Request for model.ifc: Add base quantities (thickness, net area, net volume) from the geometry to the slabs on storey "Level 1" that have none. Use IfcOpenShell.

First a look at what the model holds.

```python
import ifcopenshell
import ifcopenshell.util.element
import ifcopenshell.util.unit

model = ifcopenshell.open("model.ifc")
print(model.schema)
for unit_type in ("LENGTHUNIT", "AREAUNIT", "VOLUMEUNIT"):
    print(unit_type, ifcopenshell.util.unit.calculate_unit_scale(model, unit_type))
storey = next(s for s in model.by_type("IfcBuildingStorey") if s.Name == "Level 1")
slabs = [e for e in ifcopenshell.util.element.get_decomposition(storey) if e.is_a("IfcSlab")]
for e in sorted(slabs, key=lambda e: e.id()):
    print(e.id(), e.is_a(), e.Name, list(ifcopenshell.util.element.get_psets(e, qtos_only=True)), sep=" | ")
```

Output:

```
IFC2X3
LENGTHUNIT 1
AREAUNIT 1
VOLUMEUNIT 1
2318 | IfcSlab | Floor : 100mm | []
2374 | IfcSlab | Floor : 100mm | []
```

```python
import ifcopenshell
import ifcopenshell.api.pset
import ifcopenshell.geom
import ifcopenshell.util.element
import ifcopenshell.util.shape
import ifcopenshell.util.unit

model = ifcopenshell.open("model.ifc")
unit_scale = ifcopenshell.util.unit.calculate_unit_scale(model)
area_scale = ifcopenshell.util.unit.calculate_unit_scale(model, "AREAUNIT")
volume_scale = ifcopenshell.util.unit.calculate_unit_scale(model, "VOLUMEUNIT")
settings = ifcopenshell.geom.settings()

storey = next(s for s in model.by_type("IfcBuildingStorey") if s.Name == "Level 1")
slabs = [e for e in ifcopenshell.util.element.get_decomposition(storey) if e.is_a("IfcSlab")]

for e in sorted(slabs, key=lambda e: e.id()):
    if ifcopenshell.util.element.get_psets(e, qtos_only=True, should_inherit=False):
        continue
    # Geometry comes back in metres, in the element's own axes.
    shape = ifcopenshell.geom.create_shape(settings, e)
    values = {
        "Width": ifcopenshell.util.shape.get_z(shape.geometry) / unit_scale,
        "NetArea": ifcopenshell.util.shape.get_footprint_area(shape.geometry) / area_scale,
        "NetVolume": ifcopenshell.util.shape.get_volume(shape.geometry) / volume_scale,
    }
    qto = ifcopenshell.api.pset.add_qto(model, product=e, name="BaseQuantities")
    ifcopenshell.api.pset.edit_qto(model, qto=qto, properties=values)
    print(e.id(), {k: round(v, 3) for k, v in values.items()})

model.write("model_rev.ifc")
```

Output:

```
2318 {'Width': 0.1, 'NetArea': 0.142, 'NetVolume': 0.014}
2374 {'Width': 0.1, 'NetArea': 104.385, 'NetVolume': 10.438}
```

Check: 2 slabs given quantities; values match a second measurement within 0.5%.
